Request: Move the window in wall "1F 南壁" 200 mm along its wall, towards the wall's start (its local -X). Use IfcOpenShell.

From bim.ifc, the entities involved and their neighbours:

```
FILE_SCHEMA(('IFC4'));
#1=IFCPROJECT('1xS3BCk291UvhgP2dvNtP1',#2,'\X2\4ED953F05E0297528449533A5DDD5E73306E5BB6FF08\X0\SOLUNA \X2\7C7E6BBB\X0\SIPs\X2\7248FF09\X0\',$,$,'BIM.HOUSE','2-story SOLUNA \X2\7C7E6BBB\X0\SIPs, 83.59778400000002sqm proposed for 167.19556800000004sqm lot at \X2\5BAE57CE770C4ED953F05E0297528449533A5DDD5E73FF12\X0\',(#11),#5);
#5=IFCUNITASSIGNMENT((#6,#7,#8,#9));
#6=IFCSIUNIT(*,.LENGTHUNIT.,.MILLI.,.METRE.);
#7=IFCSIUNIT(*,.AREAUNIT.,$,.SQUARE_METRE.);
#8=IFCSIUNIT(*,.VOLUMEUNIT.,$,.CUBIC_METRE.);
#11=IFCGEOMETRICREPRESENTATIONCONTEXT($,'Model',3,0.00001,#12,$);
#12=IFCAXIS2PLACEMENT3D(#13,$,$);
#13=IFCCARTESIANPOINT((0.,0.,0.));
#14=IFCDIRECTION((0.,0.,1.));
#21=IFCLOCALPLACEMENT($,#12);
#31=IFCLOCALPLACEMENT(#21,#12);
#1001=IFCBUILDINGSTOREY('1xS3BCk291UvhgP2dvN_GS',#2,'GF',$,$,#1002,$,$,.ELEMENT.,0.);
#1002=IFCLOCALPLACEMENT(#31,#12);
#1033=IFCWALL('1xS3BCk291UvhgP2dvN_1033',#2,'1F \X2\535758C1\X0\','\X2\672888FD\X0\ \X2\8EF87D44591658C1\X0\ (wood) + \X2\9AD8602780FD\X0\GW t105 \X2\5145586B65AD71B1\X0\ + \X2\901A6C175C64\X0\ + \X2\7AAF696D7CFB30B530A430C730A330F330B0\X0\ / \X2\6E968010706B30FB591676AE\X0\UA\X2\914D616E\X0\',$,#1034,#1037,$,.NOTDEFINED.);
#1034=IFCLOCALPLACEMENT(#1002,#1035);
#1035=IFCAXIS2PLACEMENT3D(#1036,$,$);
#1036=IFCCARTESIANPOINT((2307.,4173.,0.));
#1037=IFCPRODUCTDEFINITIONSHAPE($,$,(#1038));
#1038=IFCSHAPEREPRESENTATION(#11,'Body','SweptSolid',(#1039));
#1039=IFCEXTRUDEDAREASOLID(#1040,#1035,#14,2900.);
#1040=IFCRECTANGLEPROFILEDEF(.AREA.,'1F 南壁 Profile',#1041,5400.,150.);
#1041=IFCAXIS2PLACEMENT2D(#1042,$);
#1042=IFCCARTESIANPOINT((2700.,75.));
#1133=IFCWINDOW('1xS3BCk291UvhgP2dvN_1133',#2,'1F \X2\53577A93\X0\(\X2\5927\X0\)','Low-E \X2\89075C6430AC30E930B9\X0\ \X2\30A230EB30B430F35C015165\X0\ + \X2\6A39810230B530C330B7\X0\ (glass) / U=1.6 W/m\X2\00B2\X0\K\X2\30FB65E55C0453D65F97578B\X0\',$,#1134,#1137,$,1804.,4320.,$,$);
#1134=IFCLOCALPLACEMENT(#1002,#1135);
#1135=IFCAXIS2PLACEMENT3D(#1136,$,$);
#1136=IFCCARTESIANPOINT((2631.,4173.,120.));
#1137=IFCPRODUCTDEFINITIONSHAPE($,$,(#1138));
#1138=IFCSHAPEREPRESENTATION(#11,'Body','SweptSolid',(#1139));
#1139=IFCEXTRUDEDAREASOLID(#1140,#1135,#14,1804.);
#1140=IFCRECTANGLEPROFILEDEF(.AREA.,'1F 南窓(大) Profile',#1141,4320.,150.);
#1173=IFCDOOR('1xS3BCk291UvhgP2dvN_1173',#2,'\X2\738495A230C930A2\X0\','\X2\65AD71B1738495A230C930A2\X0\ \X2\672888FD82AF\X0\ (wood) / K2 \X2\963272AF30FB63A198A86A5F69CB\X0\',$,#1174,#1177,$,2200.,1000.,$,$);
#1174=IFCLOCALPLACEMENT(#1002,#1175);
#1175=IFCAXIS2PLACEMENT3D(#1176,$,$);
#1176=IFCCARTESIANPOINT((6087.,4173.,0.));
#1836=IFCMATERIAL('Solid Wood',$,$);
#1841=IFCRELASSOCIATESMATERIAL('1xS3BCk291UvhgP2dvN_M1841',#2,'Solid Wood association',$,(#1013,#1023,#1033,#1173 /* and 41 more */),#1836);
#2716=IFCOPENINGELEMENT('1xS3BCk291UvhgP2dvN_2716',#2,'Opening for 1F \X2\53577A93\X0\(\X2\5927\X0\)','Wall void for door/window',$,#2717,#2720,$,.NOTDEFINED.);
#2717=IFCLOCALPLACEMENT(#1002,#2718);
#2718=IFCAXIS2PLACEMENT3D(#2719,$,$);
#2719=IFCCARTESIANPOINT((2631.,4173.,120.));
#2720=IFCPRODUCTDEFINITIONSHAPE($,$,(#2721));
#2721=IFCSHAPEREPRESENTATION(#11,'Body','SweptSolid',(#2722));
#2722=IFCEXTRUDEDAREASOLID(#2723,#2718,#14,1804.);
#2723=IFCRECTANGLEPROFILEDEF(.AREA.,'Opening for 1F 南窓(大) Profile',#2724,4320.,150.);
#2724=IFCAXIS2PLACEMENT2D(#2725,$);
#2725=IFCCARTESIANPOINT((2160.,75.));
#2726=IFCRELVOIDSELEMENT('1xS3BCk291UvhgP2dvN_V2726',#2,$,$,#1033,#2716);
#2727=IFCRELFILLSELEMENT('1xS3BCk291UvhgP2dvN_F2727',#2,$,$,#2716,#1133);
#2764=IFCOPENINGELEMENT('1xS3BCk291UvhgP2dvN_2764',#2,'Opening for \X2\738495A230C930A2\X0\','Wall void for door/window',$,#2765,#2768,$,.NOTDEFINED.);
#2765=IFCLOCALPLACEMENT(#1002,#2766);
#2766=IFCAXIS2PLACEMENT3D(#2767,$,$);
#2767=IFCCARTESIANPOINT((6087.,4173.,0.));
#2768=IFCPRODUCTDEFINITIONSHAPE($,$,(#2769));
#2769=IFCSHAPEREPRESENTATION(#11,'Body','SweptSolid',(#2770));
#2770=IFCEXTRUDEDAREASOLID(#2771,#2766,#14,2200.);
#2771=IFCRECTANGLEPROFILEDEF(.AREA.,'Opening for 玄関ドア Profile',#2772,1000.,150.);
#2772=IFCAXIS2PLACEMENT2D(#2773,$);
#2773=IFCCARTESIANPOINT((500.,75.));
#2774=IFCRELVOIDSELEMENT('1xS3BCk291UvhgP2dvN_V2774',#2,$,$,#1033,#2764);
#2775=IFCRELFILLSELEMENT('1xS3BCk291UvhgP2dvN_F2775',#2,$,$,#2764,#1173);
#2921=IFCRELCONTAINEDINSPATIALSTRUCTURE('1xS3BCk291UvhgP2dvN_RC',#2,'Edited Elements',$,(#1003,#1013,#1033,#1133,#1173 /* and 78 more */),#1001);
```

```python
import ifcopenshell
import ifcopenshell.api.geometry
import ifcopenshell.util.placement
import ifcopenshell.util.unit

model = ifcopenshell.open("bim.ifc")
unit_scale = ifcopenshell.util.unit.calculate_unit_scale(model)

window = model.by_guid("1xS3BCk291UvhgP2dvN_1133")
opening = window.FillsVoids[0].RelatingOpeningElement
wall = opening.VoidsElements[0].RelatingBuildingElement

wall_matrix = ifcopenshell.util.placement.get_local_placement(wall.ObjectPlacement)
shift = wall_matrix[:3, 0] * -0.2 / unit_scale
before = ifcopenshell.util.placement.get_local_placement(window.ObjectPlacement)[:3, 3].copy()

# The window is not placed relative to its opening, so move both.
for product in (opening, window):
    matrix = ifcopenshell.util.placement.get_local_placement(product.ObjectPlacement)
    matrix[:3, 3] += shift
    ifcopenshell.api.geometry.edit_object_placement(model, product=product, matrix=matrix, is_si=False)

after = ifcopenshell.util.placement.get_local_placement(window.ObjectPlacement)[:3, 3]
print("window moved by", (after - before).round(3) + 0.0)

model.write("bim_edited.ifc")
```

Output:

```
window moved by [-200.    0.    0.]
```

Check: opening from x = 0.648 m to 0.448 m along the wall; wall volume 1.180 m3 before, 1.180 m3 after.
